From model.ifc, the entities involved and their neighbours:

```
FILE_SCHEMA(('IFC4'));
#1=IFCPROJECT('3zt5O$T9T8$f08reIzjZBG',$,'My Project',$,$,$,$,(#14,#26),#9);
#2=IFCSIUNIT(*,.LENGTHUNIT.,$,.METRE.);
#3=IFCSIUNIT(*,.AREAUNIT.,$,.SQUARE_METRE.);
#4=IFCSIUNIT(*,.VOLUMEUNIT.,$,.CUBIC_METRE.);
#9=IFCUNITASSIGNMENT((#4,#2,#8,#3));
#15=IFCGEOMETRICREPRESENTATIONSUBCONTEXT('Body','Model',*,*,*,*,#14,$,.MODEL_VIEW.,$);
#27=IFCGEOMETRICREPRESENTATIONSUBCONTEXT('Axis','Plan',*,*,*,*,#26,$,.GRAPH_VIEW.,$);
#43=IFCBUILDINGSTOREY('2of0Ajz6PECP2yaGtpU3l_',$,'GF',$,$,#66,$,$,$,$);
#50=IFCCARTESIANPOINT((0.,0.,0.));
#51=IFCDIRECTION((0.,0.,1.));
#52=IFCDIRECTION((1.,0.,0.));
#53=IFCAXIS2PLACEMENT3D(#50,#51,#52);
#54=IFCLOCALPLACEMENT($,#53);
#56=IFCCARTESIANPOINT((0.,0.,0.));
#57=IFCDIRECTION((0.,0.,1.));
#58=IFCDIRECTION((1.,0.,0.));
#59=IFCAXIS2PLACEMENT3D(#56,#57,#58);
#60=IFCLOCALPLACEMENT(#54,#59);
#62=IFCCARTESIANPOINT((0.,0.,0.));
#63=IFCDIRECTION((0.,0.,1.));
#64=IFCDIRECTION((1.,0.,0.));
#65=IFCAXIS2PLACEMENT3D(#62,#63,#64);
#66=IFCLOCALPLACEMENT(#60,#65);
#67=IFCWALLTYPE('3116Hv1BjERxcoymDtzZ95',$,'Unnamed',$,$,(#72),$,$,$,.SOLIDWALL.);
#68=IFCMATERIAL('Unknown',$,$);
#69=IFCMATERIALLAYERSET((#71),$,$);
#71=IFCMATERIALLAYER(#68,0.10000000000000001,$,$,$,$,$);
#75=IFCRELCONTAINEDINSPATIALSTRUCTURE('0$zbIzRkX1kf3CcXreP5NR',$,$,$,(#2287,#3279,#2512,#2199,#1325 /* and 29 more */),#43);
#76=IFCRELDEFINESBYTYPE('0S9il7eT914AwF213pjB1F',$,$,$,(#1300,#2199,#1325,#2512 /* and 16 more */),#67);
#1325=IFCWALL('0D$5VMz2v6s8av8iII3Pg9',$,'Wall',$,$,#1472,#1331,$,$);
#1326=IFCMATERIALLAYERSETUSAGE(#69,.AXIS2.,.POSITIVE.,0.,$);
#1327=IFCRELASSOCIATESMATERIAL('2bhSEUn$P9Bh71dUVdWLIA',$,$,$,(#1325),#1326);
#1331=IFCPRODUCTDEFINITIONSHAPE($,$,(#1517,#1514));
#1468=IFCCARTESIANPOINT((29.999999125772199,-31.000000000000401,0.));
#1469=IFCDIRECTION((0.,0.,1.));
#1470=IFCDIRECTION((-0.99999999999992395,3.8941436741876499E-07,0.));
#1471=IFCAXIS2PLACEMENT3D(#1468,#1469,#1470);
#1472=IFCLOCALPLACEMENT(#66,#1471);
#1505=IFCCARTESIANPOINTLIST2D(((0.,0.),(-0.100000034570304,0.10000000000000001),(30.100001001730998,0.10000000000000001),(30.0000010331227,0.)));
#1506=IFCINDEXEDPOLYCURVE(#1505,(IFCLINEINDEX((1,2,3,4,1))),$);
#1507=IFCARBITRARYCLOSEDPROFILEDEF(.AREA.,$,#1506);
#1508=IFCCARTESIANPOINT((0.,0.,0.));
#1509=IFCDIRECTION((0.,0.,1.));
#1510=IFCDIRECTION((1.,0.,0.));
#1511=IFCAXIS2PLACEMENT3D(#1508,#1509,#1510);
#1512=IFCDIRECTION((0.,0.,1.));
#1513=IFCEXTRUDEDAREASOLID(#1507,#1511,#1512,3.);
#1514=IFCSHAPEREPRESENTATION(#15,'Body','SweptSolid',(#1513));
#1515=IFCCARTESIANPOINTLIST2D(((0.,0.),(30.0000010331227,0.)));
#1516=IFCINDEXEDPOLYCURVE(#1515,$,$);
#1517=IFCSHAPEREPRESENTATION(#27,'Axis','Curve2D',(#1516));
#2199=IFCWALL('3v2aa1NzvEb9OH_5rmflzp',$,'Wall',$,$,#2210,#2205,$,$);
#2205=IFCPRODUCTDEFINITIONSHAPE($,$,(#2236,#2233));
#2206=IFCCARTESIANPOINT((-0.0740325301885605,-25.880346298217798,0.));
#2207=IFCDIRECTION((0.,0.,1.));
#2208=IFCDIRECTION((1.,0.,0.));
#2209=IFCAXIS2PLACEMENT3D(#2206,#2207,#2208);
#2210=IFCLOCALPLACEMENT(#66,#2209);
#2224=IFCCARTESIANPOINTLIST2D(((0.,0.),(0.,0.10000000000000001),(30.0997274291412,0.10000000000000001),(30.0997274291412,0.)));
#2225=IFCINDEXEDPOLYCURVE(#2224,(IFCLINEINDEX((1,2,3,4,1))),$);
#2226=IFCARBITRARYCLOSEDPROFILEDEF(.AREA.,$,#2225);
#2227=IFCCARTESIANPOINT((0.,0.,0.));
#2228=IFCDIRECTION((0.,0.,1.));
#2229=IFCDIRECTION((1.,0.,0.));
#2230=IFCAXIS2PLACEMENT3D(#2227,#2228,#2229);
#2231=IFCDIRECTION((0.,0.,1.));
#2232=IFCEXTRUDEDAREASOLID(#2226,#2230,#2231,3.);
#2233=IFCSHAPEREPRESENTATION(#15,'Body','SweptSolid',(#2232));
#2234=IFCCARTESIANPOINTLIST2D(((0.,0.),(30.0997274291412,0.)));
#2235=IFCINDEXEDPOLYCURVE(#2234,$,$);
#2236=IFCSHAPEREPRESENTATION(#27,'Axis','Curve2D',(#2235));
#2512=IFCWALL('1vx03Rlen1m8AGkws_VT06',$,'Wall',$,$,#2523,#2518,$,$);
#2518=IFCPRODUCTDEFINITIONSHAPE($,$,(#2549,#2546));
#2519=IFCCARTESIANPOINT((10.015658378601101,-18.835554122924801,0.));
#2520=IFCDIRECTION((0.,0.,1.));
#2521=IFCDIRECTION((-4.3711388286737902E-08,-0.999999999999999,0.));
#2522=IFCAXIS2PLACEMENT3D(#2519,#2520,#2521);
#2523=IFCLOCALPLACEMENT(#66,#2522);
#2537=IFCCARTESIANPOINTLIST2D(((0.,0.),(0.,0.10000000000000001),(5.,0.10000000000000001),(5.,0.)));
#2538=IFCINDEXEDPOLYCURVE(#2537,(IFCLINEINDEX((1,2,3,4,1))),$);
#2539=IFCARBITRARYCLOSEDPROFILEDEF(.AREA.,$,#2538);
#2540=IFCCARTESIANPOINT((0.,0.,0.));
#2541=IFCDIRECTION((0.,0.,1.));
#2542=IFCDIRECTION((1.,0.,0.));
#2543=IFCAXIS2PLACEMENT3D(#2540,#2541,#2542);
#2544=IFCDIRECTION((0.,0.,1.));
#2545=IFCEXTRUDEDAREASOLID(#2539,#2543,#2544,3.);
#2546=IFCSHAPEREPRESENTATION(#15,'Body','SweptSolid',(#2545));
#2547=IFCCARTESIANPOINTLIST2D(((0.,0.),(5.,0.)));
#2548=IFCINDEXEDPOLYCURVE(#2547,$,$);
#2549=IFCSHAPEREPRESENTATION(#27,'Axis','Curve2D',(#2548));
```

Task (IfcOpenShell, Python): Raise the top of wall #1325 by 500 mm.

```python
import ifcopenshell
import ifcopenshell.geom
import ifcopenshell.util.representation
import ifcopenshell.util.shape

model = ifcopenshell.open("model.ifc")
settings = ifcopenshell.geom.settings()


def volume(element):
    """Net volume in cubic metres, openings subtracted."""
    shape = ifcopenshell.geom.create_shape(settings, element)
    return ifcopenshell.util.shape.get_volume(shape.geometry)


wall = model.by_guid("0D$5VMz2v6s8av8iII3Pg9")
before = volume(wall)

body = ifcopenshell.util.representation.get_representation(wall, "Model", "Body")
solid = body.Items[0]
old_height = solid.Depth
solid.Depth += 0.5
after = volume(wall)

print(f"height {old_height:g} -> {solid.Depth:g}, volume {before:.3f} -> {after:.3f} m3")

model.write("model_v2.ifc")
```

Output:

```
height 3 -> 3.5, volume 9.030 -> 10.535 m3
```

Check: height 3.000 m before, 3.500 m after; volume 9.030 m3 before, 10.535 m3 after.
